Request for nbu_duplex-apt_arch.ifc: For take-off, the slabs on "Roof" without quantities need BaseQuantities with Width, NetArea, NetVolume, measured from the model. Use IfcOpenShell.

First a look at what the model holds.

```python
import ifcopenshell
import ifcopenshell.util.element
import ifcopenshell.util.unit

model = ifcopenshell.open("nbu_duplex-apt_arch.ifc")
print(model.schema)
for unit_type in ("LENGTHUNIT", "AREAUNIT", "VOLUMEUNIT"):
    print(unit_type, ifcopenshell.util.unit.calculate_unit_scale(model, unit_type))
storey = next(s for s in model.by_type("IfcBuildingStorey") if s.Name == "Roof")
slabs = [e for e in ifcopenshell.util.element.get_decomposition(storey) if e.is_a("IfcSlab")]
for e in sorted(slabs, key=lambda e: e.id()):
    print(e.id(), e.is_a(), e.Name, list(ifcopenshell.util.element.get_psets(e, qtos_only=True)), sep=" | ")
```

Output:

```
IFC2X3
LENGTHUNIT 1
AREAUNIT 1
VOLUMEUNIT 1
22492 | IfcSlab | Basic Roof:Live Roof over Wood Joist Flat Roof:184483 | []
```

```python
import ifcopenshell
import ifcopenshell.api.pset
import ifcopenshell.geom
import ifcopenshell.util.element
import ifcopenshell.util.shape
import ifcopenshell.util.unit

model = ifcopenshell.open("nbu_duplex-apt_arch.ifc")
unit_scale = ifcopenshell.util.unit.calculate_unit_scale(model)
area_scale = ifcopenshell.util.unit.calculate_unit_scale(model, "AREAUNIT")
volume_scale = ifcopenshell.util.unit.calculate_unit_scale(model, "VOLUMEUNIT")
settings = ifcopenshell.geom.settings()

storey = next(s for s in model.by_type("IfcBuildingStorey") if s.Name == "Roof")
slabs = [e for e in ifcopenshell.util.element.get_decomposition(storey) if e.is_a("IfcSlab")]

for e in sorted(slabs, key=lambda e: e.id()):
    if ifcopenshell.util.element.get_psets(e, qtos_only=True, should_inherit=False):
        continue
    # Geometry comes back in metres, in the element's own axes.
    shape = ifcopenshell.geom.create_shape(settings, e)
    values = {
        "Width": ifcopenshell.util.shape.get_z(shape.geometry) / unit_scale,
        "NetArea": ifcopenshell.util.shape.get_footprint_area(shape.geometry) / area_scale,
        "NetVolume": ifcopenshell.util.shape.get_volume(shape.geometry) / volume_scale,
    }
    qto = ifcopenshell.api.pset.add_qto(model, product=e, name="BaseQuantities")
    ifcopenshell.api.pset.edit_qto(model, qto=qto, properties=values)
    print(e.id(), {k: round(v, 3) for k, v in values.items()})

model.write("nbu_duplex-apt_arch-out.ifc")
```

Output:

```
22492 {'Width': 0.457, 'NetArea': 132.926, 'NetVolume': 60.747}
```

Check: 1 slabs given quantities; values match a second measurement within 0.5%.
